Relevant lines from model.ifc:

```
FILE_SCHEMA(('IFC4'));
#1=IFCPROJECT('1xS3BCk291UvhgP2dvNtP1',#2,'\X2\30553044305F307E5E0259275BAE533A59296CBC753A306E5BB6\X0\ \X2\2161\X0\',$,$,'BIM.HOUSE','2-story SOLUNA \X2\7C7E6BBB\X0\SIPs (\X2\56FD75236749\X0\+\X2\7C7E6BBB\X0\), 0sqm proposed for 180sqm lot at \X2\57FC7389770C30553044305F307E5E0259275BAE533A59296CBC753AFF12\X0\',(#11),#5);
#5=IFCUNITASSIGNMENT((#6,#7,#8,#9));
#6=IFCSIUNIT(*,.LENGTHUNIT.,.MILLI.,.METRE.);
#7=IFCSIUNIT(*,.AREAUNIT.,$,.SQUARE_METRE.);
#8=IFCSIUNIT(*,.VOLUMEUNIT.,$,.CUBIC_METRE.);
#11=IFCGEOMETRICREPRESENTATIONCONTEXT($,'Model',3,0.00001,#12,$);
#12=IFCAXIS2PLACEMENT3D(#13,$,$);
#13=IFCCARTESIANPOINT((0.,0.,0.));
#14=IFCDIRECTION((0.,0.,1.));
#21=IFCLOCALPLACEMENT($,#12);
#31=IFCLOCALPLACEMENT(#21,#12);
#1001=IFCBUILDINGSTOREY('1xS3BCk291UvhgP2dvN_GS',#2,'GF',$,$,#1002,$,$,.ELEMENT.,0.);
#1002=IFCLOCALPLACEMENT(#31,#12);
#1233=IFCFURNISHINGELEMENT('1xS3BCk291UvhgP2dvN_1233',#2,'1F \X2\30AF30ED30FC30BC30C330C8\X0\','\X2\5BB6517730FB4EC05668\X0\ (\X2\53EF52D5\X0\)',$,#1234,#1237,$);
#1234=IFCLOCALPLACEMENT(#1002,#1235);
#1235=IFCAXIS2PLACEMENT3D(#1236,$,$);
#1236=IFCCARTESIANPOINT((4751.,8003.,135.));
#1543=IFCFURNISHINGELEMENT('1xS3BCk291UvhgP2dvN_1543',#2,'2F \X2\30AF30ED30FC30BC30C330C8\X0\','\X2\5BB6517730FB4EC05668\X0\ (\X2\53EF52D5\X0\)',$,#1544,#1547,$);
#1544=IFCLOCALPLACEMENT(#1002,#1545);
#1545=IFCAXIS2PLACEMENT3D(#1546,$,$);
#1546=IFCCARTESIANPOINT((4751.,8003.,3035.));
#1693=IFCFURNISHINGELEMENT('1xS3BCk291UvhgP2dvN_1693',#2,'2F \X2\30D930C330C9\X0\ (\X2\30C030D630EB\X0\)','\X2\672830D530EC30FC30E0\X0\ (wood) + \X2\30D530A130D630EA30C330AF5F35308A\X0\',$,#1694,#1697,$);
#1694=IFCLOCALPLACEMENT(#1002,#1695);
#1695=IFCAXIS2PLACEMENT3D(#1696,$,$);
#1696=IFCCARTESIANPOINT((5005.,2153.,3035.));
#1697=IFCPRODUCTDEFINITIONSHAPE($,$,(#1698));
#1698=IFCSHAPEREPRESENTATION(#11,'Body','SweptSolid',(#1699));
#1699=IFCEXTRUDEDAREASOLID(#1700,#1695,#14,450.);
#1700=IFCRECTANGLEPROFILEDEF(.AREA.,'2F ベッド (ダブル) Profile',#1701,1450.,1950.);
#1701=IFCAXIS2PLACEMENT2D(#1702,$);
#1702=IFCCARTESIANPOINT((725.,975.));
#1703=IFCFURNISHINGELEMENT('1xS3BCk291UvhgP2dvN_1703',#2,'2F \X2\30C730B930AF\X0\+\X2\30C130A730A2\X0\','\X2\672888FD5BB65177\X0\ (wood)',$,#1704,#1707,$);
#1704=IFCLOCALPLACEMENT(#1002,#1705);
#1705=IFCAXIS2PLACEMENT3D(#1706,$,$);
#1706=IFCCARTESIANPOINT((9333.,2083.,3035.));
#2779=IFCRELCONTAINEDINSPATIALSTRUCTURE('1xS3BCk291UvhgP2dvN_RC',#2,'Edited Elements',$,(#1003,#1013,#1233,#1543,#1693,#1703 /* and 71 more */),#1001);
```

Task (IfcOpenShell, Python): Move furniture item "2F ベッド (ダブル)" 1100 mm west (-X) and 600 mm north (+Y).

```python
import ifcopenshell
import ifcopenshell.api.geometry
import ifcopenshell.util.placement
import ifcopenshell.util.unit

model = ifcopenshell.open("model.ifc")
unit_scale = ifcopenshell.util.unit.calculate_unit_scale(model)

item = model.by_guid("1xS3BCk291UvhgP2dvN_1693")
matrix = ifcopenshell.util.placement.get_local_placement(item.ObjectPlacement)
matrix[0, 3] -= 1.1 / unit_scale
matrix[1, 3] += 0.6 / unit_scale
ifcopenshell.api.geometry.edit_object_placement(model, product=item, matrix=matrix, is_si=False)

print(ifcopenshell.util.placement.get_local_placement(item.ObjectPlacement).round(3) + 0.0)

model.write("model-out.ifc")
```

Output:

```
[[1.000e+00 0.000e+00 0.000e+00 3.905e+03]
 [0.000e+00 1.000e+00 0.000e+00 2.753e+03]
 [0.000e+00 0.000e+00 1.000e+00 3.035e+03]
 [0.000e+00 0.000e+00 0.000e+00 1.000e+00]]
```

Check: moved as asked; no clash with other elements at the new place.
